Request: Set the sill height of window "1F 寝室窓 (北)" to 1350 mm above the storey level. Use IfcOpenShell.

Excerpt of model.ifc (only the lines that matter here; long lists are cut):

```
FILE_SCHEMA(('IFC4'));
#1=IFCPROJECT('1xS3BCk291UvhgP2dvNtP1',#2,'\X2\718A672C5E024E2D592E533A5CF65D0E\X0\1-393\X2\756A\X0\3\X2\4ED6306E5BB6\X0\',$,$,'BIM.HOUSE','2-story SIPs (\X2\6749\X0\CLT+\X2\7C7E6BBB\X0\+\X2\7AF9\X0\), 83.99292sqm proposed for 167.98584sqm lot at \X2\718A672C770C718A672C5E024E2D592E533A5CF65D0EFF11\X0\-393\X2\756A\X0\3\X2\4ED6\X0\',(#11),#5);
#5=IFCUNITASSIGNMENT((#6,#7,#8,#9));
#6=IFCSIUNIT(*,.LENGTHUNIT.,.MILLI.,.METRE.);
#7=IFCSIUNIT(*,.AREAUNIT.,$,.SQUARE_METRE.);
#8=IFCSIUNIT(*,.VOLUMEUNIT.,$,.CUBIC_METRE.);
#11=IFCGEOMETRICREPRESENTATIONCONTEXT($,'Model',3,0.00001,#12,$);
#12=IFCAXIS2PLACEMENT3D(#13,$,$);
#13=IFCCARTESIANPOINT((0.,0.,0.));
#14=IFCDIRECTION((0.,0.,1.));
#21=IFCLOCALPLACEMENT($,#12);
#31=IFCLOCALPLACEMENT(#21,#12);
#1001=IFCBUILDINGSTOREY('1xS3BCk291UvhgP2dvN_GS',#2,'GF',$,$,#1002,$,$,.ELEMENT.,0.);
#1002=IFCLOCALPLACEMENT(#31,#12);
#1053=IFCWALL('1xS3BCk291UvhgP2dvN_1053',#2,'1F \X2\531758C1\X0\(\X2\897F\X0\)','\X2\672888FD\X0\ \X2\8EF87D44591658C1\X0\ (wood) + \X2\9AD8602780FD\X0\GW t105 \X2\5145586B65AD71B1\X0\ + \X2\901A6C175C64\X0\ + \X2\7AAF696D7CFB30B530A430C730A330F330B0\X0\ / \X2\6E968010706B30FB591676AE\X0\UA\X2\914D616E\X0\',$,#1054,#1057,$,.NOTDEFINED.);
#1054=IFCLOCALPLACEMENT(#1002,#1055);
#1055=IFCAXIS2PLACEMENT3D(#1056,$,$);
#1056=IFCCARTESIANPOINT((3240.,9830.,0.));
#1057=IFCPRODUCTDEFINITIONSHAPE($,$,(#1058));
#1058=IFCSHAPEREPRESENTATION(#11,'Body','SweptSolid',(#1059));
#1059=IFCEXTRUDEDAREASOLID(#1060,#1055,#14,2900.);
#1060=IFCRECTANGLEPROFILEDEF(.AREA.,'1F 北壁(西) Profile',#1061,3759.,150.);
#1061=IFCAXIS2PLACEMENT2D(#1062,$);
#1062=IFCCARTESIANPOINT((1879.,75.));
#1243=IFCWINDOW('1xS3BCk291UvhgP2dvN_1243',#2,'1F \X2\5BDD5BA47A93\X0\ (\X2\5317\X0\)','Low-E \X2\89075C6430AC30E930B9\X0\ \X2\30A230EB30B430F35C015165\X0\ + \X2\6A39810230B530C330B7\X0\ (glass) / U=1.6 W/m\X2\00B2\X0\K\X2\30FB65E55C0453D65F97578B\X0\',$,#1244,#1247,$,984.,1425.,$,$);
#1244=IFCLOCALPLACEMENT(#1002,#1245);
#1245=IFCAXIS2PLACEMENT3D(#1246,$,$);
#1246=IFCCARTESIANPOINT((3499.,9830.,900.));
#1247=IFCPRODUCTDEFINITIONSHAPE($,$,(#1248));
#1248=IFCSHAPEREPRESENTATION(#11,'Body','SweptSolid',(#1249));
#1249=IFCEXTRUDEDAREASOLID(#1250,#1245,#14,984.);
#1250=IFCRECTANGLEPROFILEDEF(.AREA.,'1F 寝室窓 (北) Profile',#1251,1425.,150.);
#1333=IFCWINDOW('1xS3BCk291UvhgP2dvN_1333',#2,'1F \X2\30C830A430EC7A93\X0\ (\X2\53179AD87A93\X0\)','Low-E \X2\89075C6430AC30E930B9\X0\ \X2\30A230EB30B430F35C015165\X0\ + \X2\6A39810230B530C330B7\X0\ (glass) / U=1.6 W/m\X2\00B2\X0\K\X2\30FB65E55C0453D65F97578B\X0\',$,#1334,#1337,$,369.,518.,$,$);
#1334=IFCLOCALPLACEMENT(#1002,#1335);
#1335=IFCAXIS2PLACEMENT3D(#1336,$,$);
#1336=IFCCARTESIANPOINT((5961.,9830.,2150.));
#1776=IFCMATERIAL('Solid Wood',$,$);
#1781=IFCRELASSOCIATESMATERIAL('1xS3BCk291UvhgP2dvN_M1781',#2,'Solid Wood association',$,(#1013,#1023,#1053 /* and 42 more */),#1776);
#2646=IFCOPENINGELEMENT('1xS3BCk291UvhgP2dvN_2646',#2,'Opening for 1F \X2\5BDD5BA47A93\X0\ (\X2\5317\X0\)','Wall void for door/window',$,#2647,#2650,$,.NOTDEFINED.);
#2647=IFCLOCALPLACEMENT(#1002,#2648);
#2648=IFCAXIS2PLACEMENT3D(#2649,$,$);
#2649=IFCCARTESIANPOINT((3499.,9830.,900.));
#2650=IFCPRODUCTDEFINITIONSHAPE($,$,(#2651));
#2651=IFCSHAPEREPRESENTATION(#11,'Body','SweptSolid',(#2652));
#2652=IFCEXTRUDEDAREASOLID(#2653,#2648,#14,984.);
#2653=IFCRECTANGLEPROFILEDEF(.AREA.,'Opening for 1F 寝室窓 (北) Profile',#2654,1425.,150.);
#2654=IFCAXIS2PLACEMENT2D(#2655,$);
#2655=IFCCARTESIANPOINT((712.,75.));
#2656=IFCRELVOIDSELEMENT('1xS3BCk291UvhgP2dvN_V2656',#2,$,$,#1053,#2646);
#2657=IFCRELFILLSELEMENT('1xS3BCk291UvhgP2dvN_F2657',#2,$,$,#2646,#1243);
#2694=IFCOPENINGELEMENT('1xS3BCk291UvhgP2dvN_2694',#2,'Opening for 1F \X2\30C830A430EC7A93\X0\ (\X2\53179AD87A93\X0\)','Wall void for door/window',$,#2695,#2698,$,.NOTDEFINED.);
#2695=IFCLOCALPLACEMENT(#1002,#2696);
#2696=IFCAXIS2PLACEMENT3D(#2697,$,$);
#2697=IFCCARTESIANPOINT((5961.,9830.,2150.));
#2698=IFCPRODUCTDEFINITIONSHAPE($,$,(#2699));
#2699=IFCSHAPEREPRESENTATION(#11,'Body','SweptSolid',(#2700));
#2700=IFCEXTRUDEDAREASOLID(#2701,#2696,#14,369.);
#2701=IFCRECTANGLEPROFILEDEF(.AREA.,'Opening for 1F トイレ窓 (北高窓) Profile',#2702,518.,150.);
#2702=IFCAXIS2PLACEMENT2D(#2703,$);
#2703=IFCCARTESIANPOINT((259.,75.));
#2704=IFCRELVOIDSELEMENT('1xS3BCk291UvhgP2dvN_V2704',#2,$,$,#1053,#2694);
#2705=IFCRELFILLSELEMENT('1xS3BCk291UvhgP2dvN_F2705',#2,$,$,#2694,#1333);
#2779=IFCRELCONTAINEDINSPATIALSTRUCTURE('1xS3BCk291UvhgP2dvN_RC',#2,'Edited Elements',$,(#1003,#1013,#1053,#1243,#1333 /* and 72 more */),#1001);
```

```python
import numpy as np
import ifcopenshell
import ifcopenshell.api.geometry
import ifcopenshell.geom
import ifcopenshell.util.element
import ifcopenshell.util.placement
import ifcopenshell.util.shape
import ifcopenshell.util.unit

model = ifcopenshell.open("model.ifc")
unit_scale = ifcopenshell.util.unit.calculate_unit_scale(model)

window = model.by_guid("1xS3BCk291UvhgP2dvN_1243")
opening = window.FillsVoids[0].RelatingOpeningElement
storey = ifcopenshell.util.element.get_container(window, ifc_class="IfcBuildingStorey")
level = ifcopenshell.util.placement.get_local_placement(storey.ObjectPlacement)[2, 3]

# The opening's origin need not be at the sill, so measure its lowest point.
shape = ifcopenshell.geom.create_shape(ifcopenshell.geom.settings(), opening)
bottom = ifcopenshell.util.shape.get_shape_bottom_elevation(shape, shape.geometry) / unit_scale
dz = level + 1350.0 - bottom

shift = np.array([0.0, 0.0, dz])
# The window is not placed relative to its opening, so move both.
for product in (opening, window):
    matrix = ifcopenshell.util.placement.get_local_placement(product.ObjectPlacement)
    matrix[:3, 3] += shift
    ifcopenshell.api.geometry.edit_object_placement(model, product=product, matrix=matrix, is_si=False)

print(f"moved by {dz * unit_scale:+.3f} m")

model.write("model_updated.ifc")
```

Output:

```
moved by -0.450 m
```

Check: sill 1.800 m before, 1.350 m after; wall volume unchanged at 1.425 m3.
